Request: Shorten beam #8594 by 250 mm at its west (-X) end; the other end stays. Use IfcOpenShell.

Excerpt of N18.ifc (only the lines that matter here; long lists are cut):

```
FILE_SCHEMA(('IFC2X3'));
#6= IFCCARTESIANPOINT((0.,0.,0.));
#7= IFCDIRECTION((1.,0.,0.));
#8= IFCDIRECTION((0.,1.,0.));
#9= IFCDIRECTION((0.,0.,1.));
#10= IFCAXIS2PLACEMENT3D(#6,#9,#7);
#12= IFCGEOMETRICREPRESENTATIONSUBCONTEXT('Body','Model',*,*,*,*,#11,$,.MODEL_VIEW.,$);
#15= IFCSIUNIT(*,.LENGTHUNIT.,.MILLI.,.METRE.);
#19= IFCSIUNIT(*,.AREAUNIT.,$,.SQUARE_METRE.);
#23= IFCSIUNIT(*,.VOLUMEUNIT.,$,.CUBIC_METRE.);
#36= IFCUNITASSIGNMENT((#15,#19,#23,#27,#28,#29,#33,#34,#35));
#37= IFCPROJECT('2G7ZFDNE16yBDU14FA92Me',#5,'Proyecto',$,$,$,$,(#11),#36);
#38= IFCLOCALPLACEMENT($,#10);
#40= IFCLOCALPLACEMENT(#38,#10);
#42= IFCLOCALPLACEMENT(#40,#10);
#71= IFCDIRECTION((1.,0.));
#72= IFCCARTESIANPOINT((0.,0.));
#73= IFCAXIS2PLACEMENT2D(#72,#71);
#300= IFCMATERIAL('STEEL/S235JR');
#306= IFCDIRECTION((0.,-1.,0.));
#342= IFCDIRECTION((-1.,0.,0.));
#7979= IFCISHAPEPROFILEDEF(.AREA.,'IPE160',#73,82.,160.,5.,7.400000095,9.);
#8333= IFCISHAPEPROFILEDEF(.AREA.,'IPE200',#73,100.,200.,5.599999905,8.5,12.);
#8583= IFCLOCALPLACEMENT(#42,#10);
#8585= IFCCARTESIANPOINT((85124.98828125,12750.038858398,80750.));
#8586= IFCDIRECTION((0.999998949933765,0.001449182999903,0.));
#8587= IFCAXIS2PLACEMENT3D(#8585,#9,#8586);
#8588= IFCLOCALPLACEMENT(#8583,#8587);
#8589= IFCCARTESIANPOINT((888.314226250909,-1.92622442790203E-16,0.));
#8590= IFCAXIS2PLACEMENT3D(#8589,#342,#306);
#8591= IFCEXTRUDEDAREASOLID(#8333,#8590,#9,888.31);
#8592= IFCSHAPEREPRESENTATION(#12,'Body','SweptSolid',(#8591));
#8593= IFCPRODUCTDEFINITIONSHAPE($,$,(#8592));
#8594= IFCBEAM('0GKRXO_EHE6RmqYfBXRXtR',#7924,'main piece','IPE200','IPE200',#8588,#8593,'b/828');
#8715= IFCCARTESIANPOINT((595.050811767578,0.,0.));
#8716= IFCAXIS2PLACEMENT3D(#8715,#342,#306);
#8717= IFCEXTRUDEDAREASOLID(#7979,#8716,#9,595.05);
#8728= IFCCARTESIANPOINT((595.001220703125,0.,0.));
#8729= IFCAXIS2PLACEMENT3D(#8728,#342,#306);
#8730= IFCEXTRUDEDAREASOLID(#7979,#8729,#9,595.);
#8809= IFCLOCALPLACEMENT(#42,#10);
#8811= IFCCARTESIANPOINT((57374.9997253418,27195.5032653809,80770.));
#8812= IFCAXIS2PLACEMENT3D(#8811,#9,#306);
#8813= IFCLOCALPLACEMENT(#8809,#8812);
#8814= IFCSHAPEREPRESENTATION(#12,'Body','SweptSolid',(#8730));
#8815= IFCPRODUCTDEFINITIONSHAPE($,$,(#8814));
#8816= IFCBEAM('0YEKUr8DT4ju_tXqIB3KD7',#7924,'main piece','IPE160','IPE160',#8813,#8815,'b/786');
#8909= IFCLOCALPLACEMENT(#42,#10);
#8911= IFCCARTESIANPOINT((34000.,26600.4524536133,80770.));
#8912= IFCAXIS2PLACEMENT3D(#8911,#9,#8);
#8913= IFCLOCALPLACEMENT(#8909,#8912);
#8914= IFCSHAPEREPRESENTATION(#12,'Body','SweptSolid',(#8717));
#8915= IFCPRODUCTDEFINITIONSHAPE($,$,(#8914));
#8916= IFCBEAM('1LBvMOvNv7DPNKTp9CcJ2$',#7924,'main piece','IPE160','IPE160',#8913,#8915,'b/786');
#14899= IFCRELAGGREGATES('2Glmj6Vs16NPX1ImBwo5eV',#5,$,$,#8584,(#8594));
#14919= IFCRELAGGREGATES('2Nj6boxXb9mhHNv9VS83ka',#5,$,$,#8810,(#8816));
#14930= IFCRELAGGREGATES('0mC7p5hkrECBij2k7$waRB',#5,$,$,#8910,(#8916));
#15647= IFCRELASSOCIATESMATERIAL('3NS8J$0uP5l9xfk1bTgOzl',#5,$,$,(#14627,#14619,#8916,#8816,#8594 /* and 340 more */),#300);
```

```python
import ifcopenshell
import ifcopenshell.util.representation
import ifcopenshell.util.unit

model = ifcopenshell.open("N18.ifc")
unit_scale = ifcopenshell.util.unit.calculate_unit_scale(model)

member = model.by_id(8594)
change = -0.25 / unit_scale

# The extrusion runs towards the end named, so only its depth changes.
body = ifcopenshell.util.representation.get_representation(member, "Model", "Body")
solid = body.Items[0]
old_length = solid.Depth
solid.Depth += change

print(f"length {old_length:g} -> {solid.Depth:g}")

model.write("N18_v2.ifc")
```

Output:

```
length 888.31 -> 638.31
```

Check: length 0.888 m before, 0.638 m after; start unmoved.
